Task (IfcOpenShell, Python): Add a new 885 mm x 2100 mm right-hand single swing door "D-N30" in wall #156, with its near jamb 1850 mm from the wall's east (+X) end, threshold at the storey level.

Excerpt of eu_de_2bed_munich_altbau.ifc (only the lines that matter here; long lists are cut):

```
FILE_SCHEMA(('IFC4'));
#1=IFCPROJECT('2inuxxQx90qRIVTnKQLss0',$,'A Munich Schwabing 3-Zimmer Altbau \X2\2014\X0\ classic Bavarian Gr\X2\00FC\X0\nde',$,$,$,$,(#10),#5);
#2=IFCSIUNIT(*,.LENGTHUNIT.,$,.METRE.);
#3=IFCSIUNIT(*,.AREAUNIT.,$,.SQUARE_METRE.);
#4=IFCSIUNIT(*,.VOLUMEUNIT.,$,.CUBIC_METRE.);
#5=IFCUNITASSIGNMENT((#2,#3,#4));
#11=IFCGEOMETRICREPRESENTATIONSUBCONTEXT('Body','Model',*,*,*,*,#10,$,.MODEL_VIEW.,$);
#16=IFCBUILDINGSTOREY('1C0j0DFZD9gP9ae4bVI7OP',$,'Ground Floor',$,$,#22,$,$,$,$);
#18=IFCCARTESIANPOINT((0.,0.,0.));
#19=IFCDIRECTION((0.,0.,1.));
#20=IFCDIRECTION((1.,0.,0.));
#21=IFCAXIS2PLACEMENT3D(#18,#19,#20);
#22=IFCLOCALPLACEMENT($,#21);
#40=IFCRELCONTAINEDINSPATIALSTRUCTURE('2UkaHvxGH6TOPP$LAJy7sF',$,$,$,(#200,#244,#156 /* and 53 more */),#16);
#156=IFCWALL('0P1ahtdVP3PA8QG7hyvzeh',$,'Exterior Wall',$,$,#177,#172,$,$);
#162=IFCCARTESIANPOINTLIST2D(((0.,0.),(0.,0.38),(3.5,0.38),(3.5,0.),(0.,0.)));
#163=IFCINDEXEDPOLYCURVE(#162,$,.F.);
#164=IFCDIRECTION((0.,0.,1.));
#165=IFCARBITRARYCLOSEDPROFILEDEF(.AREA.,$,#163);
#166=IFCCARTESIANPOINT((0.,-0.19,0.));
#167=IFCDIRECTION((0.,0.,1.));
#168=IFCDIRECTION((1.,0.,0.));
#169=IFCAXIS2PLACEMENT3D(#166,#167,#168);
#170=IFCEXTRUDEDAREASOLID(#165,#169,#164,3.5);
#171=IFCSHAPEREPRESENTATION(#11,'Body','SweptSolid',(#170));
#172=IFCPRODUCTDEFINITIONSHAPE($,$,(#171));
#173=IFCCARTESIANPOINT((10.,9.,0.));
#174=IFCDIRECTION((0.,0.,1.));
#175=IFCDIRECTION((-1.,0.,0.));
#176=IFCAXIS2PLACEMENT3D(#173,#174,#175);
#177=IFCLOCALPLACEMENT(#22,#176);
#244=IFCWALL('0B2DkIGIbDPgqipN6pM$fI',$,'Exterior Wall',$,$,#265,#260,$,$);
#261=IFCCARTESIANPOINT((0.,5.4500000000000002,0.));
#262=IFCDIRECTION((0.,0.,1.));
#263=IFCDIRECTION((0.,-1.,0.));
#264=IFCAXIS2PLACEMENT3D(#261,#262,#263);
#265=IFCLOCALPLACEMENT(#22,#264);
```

```python
import numpy as np
import ifcopenshell
import ifcopenshell.api.feature
import ifcopenshell.api.geometry
import ifcopenshell.api.root
import ifcopenshell.api.spatial
import ifcopenshell.geom
import ifcopenshell.util.element
import ifcopenshell.util.placement
import ifcopenshell.util.representation
import ifcopenshell.util.shape
import ifcopenshell.util.unit

model = ifcopenshell.open("eu_de_2bed_munich_altbau.ifc")
unit_scale = ifcopenshell.util.unit.calculate_unit_scale(model)
settings = ifcopenshell.geom.settings()


def volume(element):
    """Net volume in cubic metres, openings subtracted."""
    shape = ifcopenshell.geom.create_shape(settings, element)
    return ifcopenshell.util.shape.get_volume(shape.geometry)


wall = model.by_id(156)
storey = ifcopenshell.util.element.get_container(wall, ifc_class="IfcBuildingStorey")
context = ifcopenshell.util.representation.get_context(model, "Model", "Body", "MODEL_VIEW")
before = volume(wall)

width, height, from_end, sill = 0.885, 2.1, 1.85, 0.0  # metres

# The wall runs along its own X axis, and the end named is its -X end.
wall_shape = ifcopenshell.geom.create_shape(settings, wall)
x, y, z = ifcopenshell.util.shape.get_vertices(wall_shape.geometry).T
start = x.min() + from_end
face, thickness = float(y.min()), float(y.max() - y.min())
wall_matrix = ifcopenshell.util.placement.get_local_placement(wall.ObjectPlacement)
level = ifcopenshell.util.placement.get_local_placement(storey.ObjectPlacement)[2, 3]


def in_wall(x, y):
    """Placement at x, y metres in the wall's axes, at sill height."""
    matrix = wall_matrix.copy()
    matrix[:, 3] = wall_matrix @ np.array([x / unit_scale, y / unit_scale, 0.0, 1.0])
    matrix[2, 3] = level + sill / unit_scale
    return matrix


# Opening: a box that overshoots both wall faces by 50 mm.
opening = ifcopenshell.api.root.create_entity(model, ifc_class="IfcOpeningElement", predefined_type="OPENING")
box = ifcopenshell.api.geometry.add_wall_representation(
    model, context=context, length=width, height=height, thickness=thickness + 0.1
)
ifcopenshell.api.geometry.assign_representation(model, product=opening, representation=box)
ifcopenshell.api.geometry.edit_object_placement(model, product=opening, matrix=in_wall(start, face - 0.05), is_si=False)
ifcopenshell.api.feature.add_feature(model, feature=opening, element=wall)

door = ifcopenshell.api.root.create_entity(model, ifc_class="IfcDoor", name="D-N30", predefined_type="DOOR")
door.OverallWidth, door.OverallHeight = width / unit_scale, height / unit_scale
door.OperationType = "SINGLE_SWING_RIGHT"
body = ifcopenshell.api.geometry.add_door_representation(
    model,
    context=context,
    overall_width=door.OverallWidth,
    overall_height=door.OverallHeight,
    operation_type="SINGLE_SWING_RIGHT",
    lining_properties={"LiningDepth": thickness / unit_scale, "ThresholdDepth": thickness / unit_scale},
)
ifcopenshell.api.geometry.assign_representation(model, product=door, representation=body)
ifcopenshell.api.spatial.assign_container(model, products=[door], relating_structure=storey)
ifcopenshell.api.feature.add_filling(model, opening=opening, element=door)

# The lining spans the wall, so the door starts at the wall face.
ifcopenshell.api.geometry.edit_object_placement(model, product=door, matrix=in_wall(start, face), is_si=False)

after = volume(wall)

print(f"wall volume {before:.3f} -> {after:.3f} m3")

model.write("eu_de_2bed_munich_altbau_rev.ifc")
```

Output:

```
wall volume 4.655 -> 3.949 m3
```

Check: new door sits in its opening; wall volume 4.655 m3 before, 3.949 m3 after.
